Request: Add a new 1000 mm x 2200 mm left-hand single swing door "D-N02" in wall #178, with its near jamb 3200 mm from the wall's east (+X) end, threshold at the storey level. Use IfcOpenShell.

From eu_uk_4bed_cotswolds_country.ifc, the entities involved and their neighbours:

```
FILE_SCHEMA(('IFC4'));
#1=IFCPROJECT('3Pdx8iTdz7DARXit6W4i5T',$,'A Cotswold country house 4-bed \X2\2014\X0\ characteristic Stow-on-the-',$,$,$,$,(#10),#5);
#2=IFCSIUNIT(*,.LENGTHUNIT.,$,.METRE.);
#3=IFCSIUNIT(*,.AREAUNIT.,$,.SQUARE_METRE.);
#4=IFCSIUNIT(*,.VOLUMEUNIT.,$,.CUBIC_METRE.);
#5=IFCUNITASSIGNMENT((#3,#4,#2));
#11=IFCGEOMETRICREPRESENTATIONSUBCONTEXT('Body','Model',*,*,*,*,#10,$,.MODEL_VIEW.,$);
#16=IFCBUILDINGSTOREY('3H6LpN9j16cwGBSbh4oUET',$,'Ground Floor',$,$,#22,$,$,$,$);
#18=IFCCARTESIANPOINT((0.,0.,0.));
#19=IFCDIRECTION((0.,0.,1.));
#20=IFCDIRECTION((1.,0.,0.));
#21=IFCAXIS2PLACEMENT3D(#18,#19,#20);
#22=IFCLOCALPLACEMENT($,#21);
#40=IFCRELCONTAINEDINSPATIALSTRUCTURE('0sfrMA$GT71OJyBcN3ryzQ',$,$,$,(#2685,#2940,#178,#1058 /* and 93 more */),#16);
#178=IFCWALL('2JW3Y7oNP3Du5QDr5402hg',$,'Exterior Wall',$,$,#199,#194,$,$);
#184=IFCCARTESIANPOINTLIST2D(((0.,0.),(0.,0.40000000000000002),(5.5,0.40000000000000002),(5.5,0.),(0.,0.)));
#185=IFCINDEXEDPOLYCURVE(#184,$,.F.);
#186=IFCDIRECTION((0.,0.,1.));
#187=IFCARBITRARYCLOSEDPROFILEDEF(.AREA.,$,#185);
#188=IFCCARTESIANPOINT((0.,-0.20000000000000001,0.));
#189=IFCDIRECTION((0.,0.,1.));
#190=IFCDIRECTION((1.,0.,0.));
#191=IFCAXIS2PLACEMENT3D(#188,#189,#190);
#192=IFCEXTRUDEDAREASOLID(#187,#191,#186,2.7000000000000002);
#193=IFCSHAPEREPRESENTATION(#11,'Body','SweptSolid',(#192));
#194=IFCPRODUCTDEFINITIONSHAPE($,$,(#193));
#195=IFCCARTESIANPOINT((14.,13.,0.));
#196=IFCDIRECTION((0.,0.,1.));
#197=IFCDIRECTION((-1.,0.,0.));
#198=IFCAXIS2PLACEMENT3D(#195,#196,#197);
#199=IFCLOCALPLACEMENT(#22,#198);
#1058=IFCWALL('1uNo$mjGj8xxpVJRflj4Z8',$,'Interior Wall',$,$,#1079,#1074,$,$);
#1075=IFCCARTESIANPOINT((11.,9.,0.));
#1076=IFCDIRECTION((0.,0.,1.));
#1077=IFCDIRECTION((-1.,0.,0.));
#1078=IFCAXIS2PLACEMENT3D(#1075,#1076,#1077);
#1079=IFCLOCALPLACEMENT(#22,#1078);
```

```python
import numpy as np
import ifcopenshell
import ifcopenshell.api.feature
import ifcopenshell.api.geometry
import ifcopenshell.api.root
import ifcopenshell.api.spatial
import ifcopenshell.geom
import ifcopenshell.util.element
import ifcopenshell.util.placement
import ifcopenshell.util.representation
import ifcopenshell.util.shape
import ifcopenshell.util.unit

model = ifcopenshell.open("eu_uk_4bed_cotswolds_country.ifc")
unit_scale = ifcopenshell.util.unit.calculate_unit_scale(model)
settings = ifcopenshell.geom.settings()


def volume(element):
    """Net volume in cubic metres, openings subtracted."""
    shape = ifcopenshell.geom.create_shape(settings, element)
    return ifcopenshell.util.shape.get_volume(shape.geometry)


wall = model.by_guid("2JW3Y7oNP3Du5QDr5402hg")
storey = ifcopenshell.util.element.get_container(wall, ifc_class="IfcBuildingStorey")
context = ifcopenshell.util.representation.get_context(model, "Model", "Body", "MODEL_VIEW")
before = volume(wall)

width, height, from_end, sill = 1, 2.2, 3.2, 0.0  # metres

# The wall runs along its own X axis, and the end named is its -X end.
wall_shape = ifcopenshell.geom.create_shape(settings, wall)
x, y, z = ifcopenshell.util.shape.get_vertices(wall_shape.geometry).T
start = x.min() + from_end
face, thickness = float(y.min()), float(y.max() - y.min())
wall_matrix = ifcopenshell.util.placement.get_local_placement(wall.ObjectPlacement)
level = ifcopenshell.util.placement.get_local_placement(storey.ObjectPlacement)[2, 3]


def in_wall(x, y):
    """Placement at x, y metres in the wall's axes, at sill height."""
    matrix = wall_matrix.copy()
    matrix[:, 3] = wall_matrix @ np.array([x / unit_scale, y / unit_scale, 0.0, 1.0])
    matrix[2, 3] = level + sill / unit_scale
    return matrix


# Opening: a box that overshoots both wall faces by 50 mm.
opening = ifcopenshell.api.root.create_entity(model, ifc_class="IfcOpeningElement", predefined_type="OPENING")
box = ifcopenshell.api.geometry.add_wall_representation(
    model, context=context, length=width, height=height, thickness=thickness + 0.1
)
ifcopenshell.api.geometry.assign_representation(model, product=opening, representation=box)
ifcopenshell.api.geometry.edit_object_placement(model, product=opening, matrix=in_wall(start, face - 0.05), is_si=False)
ifcopenshell.api.feature.add_feature(model, feature=opening, element=wall)

door = ifcopenshell.api.root.create_entity(model, ifc_class="IfcDoor", name="D-N02", predefined_type="DOOR")
door.OverallWidth, door.OverallHeight = width / unit_scale, height / unit_scale
door.OperationType = "SINGLE_SWING_LEFT"
body = ifcopenshell.api.geometry.add_door_representation(
    model,
    context=context,
    overall_width=door.OverallWidth,
    overall_height=door.OverallHeight,
    operation_type="SINGLE_SWING_LEFT",
    lining_properties={"LiningDepth": thickness / unit_scale, "ThresholdDepth": thickness / unit_scale},
)
ifcopenshell.api.geometry.assign_representation(model, product=door, representation=body)
ifcopenshell.api.spatial.assign_container(model, products=[door], relating_structure=storey)
ifcopenshell.api.feature.add_filling(model, opening=opening, element=door)

# The lining spans the wall, so the door starts at the wall face.
ifcopenshell.api.geometry.edit_object_placement(model, product=door, matrix=in_wall(start, face), is_si=False)

after = volume(wall)

print(f"wall volume {before:.3f} -> {after:.3f} m3")

model.write("eu_uk_4bed_cotswolds_country_edited.ifc")
```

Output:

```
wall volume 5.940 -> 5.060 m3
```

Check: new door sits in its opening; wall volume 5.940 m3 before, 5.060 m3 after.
